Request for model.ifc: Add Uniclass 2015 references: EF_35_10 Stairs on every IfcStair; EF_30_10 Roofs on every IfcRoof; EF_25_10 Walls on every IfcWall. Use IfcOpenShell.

First a look at what the model holds.

```python
import ifcopenshell

model = ifcopenshell.open("model.ifc")
print(model.schema)
print("classifications:", [c.Name for c in model.by_type("IfcClassification")])
for ifc_class in ("IfcDoor", "IfcRoof", "IfcStair", "IfcWall", "IfcWindow"):
    print(ifc_class, len(model.by_type(ifc_class)))
```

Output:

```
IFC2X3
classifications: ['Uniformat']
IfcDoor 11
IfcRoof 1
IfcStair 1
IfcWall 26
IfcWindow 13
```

```python
import ifcopenshell
import ifcopenshell.api.classification

model = ifcopenshell.open("model.ifc")

# IFC2X3 requires Source and Edition and has no link from the project to the system.
system = model.create_entity("IfcClassification", Source="NBS", Edition="2015", Name="Uniclass 2015")

codes = {
    "IfcStair": ("EF_35_10", "Stairs"),
    "IfcRoof": ("EF_30_10", "Roofs"),
    "IfcWall": ("EF_25_10", "Walls"),
}
for ifc_class, (code, name) in codes.items():
    products = model.by_type(ifc_class)
    ifcopenshell.api.classification.add_reference(
        model, products=products, classification=system, identification=code, name=name
    )
    print(code, len(products))

model.write("model_edited.ifc")
```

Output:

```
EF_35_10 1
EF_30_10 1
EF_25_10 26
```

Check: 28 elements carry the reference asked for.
